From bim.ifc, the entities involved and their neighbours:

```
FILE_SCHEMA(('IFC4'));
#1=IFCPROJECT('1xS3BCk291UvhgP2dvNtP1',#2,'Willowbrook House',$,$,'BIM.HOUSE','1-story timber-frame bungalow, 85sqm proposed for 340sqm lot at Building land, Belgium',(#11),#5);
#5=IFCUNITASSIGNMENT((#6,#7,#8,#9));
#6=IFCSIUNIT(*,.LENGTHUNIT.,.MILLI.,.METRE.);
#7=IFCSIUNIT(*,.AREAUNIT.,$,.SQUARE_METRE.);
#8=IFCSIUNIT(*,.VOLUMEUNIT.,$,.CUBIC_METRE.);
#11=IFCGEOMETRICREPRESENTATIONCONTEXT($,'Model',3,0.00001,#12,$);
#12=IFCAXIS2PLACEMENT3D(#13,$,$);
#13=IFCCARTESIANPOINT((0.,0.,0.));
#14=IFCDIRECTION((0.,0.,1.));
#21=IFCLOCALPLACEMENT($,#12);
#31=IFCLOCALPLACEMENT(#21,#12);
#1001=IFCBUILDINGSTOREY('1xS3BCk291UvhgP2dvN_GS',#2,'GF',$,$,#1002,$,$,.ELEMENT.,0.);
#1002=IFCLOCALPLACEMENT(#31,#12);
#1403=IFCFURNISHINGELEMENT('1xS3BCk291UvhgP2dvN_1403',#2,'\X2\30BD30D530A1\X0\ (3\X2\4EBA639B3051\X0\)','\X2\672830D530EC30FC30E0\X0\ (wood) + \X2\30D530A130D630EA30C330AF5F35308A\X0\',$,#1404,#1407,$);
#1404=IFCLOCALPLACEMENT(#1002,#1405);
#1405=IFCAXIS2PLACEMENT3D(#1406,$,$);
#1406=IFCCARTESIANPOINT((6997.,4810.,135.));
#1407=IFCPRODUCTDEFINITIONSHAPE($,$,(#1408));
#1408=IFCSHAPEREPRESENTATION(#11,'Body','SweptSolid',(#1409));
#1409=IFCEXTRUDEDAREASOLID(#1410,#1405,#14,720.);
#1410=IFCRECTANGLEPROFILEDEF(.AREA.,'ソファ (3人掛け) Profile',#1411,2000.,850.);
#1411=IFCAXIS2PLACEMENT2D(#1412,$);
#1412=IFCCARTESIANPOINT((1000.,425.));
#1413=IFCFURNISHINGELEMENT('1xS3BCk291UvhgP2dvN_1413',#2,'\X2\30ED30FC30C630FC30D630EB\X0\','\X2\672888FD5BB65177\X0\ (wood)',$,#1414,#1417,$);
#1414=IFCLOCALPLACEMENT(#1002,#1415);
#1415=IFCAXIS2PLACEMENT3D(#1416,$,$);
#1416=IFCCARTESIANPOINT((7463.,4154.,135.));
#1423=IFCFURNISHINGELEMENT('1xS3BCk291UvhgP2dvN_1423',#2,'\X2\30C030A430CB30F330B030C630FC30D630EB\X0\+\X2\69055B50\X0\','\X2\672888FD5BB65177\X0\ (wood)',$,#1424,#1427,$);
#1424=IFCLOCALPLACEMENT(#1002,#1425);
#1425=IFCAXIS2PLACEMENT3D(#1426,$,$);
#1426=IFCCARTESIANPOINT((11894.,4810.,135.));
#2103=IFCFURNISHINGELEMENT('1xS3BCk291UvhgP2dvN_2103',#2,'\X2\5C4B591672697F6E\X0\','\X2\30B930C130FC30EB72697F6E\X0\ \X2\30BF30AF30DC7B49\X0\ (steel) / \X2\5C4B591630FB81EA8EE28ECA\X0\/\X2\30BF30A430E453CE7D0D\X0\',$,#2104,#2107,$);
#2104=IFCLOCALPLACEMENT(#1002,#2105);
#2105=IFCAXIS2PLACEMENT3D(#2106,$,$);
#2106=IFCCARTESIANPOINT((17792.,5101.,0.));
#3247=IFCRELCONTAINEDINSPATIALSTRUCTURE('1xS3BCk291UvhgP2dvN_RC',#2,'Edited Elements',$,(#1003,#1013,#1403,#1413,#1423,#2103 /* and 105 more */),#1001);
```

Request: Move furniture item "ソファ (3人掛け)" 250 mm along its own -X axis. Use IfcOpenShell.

```python
import ifcopenshell
import ifcopenshell.api.geometry
import ifcopenshell.util.placement

model = ifcopenshell.open("bim.ifc")

item = model.by_guid("1xS3BCk291UvhgP2dvN_1403")
matrix = ifcopenshell.util.placement.get_local_placement(item.ObjectPlacement)
matrix[:3, 3] -= matrix[:3, 0] * 250.0
ifcopenshell.api.geometry.edit_object_placement(model, product=item, matrix=matrix, is_si=False)

print(ifcopenshell.util.placement.get_local_placement(item.ObjectPlacement).round(3) + 0.0)

model.write("bim_rev.ifc")
```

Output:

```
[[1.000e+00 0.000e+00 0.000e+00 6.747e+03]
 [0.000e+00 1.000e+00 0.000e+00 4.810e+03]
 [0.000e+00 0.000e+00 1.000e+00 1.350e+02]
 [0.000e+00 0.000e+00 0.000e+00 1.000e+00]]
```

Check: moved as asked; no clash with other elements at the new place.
